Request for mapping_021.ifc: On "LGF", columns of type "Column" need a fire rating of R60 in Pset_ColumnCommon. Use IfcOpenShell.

First a look at what the model holds.

```python
import ifcopenshell
import ifcopenshell.util.element

model = ifcopenshell.open("mapping_021.ifc")
print(model.schema)
storey = next(s for s in model.by_type("IfcBuildingStorey") if s.Name == "LGF")
columns = [e for e in ifcopenshell.util.element.get_decomposition(storey) if e.is_a("IfcColumn")]
seen = {}
for e in columns:
    element_type = ifcopenshell.util.element.get_type(e)
    key = (element_type.Name if element_type != e and element_type else None, ifcopenshell.util.element.get_pset(e, "Pset_ColumnCommon", "FireRating"))
    seen[key] = seen.get(key, 0) + 1
for (name, value), count in sorted(seen.items(), key=str):
    print(count, "x", name, "|", value)
```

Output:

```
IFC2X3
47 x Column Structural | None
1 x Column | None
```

```python
import ifcopenshell
import ifcopenshell.api.pset
import ifcopenshell.util.element

model = ifcopenshell.open("mapping_021.ifc")

storey = next(s for s in model.by_type("IfcBuildingStorey") if s.Name == "LGF")
columns = [e for e in ifcopenshell.util.element.get_decomposition(storey) if e.is_a("IfcColumn")]

count = 0
for e in columns:
    element_type = ifcopenshell.util.element.get_type(e)
    if element_type in (None, e) or element_type.Name != "Column":
        continue
    # add_pset returns the element's existing set when there is one.
    pset = ifcopenshell.api.pset.add_pset(model, product=e, name="Pset_ColumnCommon")
    ifcopenshell.api.pset.edit_pset(model, pset=pset, properties={"FireRating": "R60"})
    count += 1

print(count, "columns updated")

model.write("mapping_021_updated.ifc")
```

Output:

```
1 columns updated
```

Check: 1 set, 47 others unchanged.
